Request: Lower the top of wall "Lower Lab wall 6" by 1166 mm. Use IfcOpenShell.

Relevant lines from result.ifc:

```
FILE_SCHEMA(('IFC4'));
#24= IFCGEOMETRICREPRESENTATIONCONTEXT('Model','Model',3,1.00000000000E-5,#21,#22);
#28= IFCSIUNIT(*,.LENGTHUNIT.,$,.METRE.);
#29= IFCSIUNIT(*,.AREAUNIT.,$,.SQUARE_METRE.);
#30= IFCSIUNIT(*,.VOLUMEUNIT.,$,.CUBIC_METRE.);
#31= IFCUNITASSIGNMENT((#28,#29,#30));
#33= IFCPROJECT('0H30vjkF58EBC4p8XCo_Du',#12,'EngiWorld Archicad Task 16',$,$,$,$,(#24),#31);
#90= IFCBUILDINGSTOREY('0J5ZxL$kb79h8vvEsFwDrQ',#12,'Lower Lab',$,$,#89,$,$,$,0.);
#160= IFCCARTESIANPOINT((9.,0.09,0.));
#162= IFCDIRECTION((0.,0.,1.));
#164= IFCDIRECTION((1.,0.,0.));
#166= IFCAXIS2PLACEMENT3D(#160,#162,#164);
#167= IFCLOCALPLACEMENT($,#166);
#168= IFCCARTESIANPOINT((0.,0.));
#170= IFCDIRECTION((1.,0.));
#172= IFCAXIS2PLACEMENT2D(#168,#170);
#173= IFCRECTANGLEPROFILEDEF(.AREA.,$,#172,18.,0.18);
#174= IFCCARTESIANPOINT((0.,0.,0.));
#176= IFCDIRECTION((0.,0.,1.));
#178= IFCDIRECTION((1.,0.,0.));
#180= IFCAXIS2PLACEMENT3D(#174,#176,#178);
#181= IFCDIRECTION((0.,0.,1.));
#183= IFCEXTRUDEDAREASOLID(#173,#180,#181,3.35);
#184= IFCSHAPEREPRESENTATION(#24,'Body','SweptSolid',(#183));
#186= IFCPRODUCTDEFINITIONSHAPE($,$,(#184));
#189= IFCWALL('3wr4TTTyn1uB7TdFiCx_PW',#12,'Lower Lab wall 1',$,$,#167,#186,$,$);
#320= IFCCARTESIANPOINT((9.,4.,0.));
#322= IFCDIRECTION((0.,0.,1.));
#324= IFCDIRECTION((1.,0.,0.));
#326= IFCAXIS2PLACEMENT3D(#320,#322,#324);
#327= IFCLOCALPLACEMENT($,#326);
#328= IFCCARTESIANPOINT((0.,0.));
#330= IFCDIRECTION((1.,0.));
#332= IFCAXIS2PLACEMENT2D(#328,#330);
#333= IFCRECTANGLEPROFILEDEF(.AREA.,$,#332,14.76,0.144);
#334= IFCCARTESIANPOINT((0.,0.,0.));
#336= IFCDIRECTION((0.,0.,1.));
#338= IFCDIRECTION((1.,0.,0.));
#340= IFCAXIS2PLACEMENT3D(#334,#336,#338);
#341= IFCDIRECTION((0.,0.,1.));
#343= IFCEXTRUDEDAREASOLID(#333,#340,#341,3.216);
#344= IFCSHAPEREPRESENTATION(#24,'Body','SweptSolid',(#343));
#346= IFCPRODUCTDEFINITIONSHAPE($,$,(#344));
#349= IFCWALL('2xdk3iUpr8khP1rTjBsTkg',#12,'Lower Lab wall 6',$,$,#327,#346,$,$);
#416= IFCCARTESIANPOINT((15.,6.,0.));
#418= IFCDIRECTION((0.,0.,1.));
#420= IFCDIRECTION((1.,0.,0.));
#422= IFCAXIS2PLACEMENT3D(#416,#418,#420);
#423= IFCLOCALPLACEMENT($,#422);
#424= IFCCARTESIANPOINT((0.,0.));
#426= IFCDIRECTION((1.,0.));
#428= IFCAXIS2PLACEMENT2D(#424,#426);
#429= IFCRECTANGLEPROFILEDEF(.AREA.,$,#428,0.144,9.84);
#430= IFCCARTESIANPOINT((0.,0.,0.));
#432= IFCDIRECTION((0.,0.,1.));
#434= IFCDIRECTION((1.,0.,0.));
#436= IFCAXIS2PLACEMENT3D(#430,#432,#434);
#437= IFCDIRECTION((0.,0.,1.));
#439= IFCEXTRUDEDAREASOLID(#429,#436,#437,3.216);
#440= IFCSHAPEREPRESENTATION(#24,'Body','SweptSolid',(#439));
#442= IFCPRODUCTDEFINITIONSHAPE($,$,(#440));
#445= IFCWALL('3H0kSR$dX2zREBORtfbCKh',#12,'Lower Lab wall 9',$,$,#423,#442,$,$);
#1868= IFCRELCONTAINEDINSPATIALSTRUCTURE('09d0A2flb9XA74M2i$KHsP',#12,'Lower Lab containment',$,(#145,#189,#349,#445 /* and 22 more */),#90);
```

```python
import ifcopenshell
import ifcopenshell.geom
import ifcopenshell.util.shape

model = ifcopenshell.open("result.ifc")
settings = ifcopenshell.geom.settings()


def volume(element):
    """Net volume in cubic metres, openings subtracted."""
    shape = ifcopenshell.geom.create_shape(settings, element)
    return ifcopenshell.util.shape.get_volume(shape.geometry)


wall = model.by_id(349)
before = volume(wall)

body = next(r for r in wall.Representation.Representations if r.RepresentationIdentifier == "Body")
solid = body.Items[0]
old_height = solid.Depth
solid.Depth -= 1.166
after = volume(wall)

print(f"height {old_height:g} -> {solid.Depth:g}, volume {before:.3f} -> {after:.3f} m3")

model.write("result_v2.ifc")
```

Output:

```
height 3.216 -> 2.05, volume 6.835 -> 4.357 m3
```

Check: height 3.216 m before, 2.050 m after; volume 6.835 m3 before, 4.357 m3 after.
